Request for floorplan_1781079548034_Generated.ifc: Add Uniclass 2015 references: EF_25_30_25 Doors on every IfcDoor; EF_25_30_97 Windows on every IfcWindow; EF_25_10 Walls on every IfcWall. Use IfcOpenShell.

First a look at what the model holds.

```python
import ifcopenshell

model = ifcopenshell.open("floorplan_1781079548034_Generated.ifc")
print(model.schema)
print("classifications:", [c.Name for c in model.by_type("IfcClassification")])
for ifc_class in ("IfcDoor", "IfcRoof", "IfcStair", "IfcWall", "IfcWindow"):
    print(ifc_class, len(model.by_type(ifc_class)))
```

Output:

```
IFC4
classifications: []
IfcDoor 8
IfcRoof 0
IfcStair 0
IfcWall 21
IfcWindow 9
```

```python
import ifcopenshell
import ifcopenshell.api.classification

model = ifcopenshell.open("floorplan_1781079548034_Generated.ifc")

system = ifcopenshell.api.classification.add_classification(model, classification="Uniclass 2015")

codes = {
    "IfcDoor": ("EF_25_30_25", "Doors"),
    "IfcWindow": ("EF_25_30_97", "Windows"),
    "IfcWall": ("EF_25_10", "Walls"),
}
for ifc_class, (code, name) in codes.items():
    products = model.by_type(ifc_class)
    ifcopenshell.api.classification.add_reference(
        model, products=products, classification=system, identification=code, name=name
    )
    print(code, len(products))

model.write("floorplan_1781079548034_Generated_v2.ifc")
```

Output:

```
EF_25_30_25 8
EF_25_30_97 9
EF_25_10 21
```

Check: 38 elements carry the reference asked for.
